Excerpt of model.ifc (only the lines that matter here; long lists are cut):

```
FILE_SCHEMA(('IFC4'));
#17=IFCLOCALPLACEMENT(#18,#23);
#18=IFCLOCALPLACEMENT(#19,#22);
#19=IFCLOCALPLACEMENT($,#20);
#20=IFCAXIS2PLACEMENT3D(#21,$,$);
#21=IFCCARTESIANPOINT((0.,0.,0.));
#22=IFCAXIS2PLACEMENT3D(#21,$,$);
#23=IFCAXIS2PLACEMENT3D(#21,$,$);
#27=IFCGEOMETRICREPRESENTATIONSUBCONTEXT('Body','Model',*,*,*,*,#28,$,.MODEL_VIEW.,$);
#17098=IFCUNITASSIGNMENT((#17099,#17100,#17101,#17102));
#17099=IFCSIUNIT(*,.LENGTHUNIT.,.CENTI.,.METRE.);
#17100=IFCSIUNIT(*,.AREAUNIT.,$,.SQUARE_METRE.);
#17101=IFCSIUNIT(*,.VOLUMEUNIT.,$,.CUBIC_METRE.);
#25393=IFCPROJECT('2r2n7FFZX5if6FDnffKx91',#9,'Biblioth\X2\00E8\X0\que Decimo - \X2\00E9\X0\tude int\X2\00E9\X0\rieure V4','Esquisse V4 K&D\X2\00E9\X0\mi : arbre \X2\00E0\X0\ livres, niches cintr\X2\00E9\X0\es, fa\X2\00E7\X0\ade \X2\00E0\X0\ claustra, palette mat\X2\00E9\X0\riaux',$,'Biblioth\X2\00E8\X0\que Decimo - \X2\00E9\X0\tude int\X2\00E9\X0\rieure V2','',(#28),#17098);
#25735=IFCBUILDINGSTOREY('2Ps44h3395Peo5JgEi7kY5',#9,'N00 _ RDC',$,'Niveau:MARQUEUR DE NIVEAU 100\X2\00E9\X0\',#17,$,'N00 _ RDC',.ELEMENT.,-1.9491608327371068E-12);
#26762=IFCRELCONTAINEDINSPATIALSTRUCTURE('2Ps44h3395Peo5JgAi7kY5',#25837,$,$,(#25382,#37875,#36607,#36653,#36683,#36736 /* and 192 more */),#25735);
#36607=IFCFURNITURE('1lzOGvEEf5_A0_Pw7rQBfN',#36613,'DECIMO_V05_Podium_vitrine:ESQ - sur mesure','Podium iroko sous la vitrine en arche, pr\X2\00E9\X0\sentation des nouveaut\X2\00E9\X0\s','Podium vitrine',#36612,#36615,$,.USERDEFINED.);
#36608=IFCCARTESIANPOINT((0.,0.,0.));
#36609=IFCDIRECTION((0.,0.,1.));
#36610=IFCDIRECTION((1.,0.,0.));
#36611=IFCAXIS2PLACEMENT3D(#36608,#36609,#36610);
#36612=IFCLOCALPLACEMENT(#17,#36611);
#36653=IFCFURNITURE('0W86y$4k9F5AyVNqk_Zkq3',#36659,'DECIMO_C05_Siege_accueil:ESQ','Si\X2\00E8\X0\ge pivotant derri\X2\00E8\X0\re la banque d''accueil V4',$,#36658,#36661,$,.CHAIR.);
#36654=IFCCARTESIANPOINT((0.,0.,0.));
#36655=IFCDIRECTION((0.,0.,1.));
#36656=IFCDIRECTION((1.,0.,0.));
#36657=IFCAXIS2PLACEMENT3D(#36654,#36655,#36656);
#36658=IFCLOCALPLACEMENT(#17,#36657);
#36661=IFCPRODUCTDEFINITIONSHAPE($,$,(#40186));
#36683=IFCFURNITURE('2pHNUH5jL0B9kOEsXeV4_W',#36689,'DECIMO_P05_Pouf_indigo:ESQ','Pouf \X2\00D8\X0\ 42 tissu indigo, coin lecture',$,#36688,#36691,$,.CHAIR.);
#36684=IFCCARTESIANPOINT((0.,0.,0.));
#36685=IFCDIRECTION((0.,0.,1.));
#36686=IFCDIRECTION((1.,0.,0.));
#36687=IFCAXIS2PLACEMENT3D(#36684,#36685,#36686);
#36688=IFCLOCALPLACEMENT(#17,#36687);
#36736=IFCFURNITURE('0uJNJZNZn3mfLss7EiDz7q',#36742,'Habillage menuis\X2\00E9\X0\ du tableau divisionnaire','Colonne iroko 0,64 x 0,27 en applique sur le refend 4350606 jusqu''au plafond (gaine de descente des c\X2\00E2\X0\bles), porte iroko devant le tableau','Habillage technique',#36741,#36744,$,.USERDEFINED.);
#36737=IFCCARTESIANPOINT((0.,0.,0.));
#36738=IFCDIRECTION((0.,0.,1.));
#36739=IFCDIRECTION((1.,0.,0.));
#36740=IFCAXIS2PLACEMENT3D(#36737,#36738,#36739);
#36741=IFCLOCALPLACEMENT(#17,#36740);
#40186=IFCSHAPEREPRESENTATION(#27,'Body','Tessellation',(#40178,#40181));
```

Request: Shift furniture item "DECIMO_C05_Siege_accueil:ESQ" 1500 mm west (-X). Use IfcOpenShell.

```python
import ifcopenshell
import ifcopenshell.api.geometry
import ifcopenshell.util.placement
import ifcopenshell.util.unit

model = ifcopenshell.open("model.ifc")
unit_scale = ifcopenshell.util.unit.calculate_unit_scale(model)

item = model.by_guid("0W86y$4k9F5AyVNqk_Zkq3")
matrix = ifcopenshell.util.placement.get_local_placement(item.ObjectPlacement)
matrix[0, 3] -= 1.5 / unit_scale
ifcopenshell.api.geometry.edit_object_placement(model, product=item, matrix=matrix, is_si=False)

print(ifcopenshell.util.placement.get_local_placement(item.ObjectPlacement).round(3) + 0.0)

model.write("model_rev.ifc")
```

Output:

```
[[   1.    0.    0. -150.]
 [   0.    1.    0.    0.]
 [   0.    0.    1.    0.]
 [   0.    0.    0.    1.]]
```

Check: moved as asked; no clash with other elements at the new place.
